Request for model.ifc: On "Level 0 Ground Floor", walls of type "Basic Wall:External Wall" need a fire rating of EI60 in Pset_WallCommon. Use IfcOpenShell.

First a look at what the model holds.

```python
import ifcopenshell
import ifcopenshell.util.element

model = ifcopenshell.open("model.ifc")
print(model.schema)
storey = next(s for s in model.by_type("IfcBuildingStorey") if s.Name == "Level 0 Ground Floor")
walls = [e for e in ifcopenshell.util.element.get_decomposition(storey) if e.is_a("IfcWall")]
seen = {}
for e in walls:
    element_type = ifcopenshell.util.element.get_type(e)
    key = (element_type.Name if element_type != e and element_type else None, ifcopenshell.util.element.get_pset(e, "Pset_WallCommon", "FireRating"))
    seen[key] = seen.get(key, 0) + 1
for (name, value), count in sorted(seen.items(), key=str):
    print(count, "x", name, "|", value)
```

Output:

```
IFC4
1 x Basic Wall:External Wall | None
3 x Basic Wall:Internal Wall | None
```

```python
import ifcopenshell
import ifcopenshell.api.pset
import ifcopenshell.util.element

model = ifcopenshell.open("model.ifc")

storey = next(s for s in model.by_type("IfcBuildingStorey") if s.Name == "Level 0 Ground Floor")
walls = [e for e in ifcopenshell.util.element.get_decomposition(storey) if e.is_a("IfcWall")]

count = 0
for e in walls:
    element_type = ifcopenshell.util.element.get_type(e)
    if element_type in (None, e) or element_type.Name != "Basic Wall:External Wall":
        continue
    # add_pset returns the element's existing set when there is one.
    pset = ifcopenshell.api.pset.add_pset(model, product=e, name="Pset_WallCommon")
    ifcopenshell.api.pset.edit_pset(model, pset=pset, properties={"FireRating": "EI60"})
    count += 1

print(count, "walls updated")

model.write("model_rev.ifc")
```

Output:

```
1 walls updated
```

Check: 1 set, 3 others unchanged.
